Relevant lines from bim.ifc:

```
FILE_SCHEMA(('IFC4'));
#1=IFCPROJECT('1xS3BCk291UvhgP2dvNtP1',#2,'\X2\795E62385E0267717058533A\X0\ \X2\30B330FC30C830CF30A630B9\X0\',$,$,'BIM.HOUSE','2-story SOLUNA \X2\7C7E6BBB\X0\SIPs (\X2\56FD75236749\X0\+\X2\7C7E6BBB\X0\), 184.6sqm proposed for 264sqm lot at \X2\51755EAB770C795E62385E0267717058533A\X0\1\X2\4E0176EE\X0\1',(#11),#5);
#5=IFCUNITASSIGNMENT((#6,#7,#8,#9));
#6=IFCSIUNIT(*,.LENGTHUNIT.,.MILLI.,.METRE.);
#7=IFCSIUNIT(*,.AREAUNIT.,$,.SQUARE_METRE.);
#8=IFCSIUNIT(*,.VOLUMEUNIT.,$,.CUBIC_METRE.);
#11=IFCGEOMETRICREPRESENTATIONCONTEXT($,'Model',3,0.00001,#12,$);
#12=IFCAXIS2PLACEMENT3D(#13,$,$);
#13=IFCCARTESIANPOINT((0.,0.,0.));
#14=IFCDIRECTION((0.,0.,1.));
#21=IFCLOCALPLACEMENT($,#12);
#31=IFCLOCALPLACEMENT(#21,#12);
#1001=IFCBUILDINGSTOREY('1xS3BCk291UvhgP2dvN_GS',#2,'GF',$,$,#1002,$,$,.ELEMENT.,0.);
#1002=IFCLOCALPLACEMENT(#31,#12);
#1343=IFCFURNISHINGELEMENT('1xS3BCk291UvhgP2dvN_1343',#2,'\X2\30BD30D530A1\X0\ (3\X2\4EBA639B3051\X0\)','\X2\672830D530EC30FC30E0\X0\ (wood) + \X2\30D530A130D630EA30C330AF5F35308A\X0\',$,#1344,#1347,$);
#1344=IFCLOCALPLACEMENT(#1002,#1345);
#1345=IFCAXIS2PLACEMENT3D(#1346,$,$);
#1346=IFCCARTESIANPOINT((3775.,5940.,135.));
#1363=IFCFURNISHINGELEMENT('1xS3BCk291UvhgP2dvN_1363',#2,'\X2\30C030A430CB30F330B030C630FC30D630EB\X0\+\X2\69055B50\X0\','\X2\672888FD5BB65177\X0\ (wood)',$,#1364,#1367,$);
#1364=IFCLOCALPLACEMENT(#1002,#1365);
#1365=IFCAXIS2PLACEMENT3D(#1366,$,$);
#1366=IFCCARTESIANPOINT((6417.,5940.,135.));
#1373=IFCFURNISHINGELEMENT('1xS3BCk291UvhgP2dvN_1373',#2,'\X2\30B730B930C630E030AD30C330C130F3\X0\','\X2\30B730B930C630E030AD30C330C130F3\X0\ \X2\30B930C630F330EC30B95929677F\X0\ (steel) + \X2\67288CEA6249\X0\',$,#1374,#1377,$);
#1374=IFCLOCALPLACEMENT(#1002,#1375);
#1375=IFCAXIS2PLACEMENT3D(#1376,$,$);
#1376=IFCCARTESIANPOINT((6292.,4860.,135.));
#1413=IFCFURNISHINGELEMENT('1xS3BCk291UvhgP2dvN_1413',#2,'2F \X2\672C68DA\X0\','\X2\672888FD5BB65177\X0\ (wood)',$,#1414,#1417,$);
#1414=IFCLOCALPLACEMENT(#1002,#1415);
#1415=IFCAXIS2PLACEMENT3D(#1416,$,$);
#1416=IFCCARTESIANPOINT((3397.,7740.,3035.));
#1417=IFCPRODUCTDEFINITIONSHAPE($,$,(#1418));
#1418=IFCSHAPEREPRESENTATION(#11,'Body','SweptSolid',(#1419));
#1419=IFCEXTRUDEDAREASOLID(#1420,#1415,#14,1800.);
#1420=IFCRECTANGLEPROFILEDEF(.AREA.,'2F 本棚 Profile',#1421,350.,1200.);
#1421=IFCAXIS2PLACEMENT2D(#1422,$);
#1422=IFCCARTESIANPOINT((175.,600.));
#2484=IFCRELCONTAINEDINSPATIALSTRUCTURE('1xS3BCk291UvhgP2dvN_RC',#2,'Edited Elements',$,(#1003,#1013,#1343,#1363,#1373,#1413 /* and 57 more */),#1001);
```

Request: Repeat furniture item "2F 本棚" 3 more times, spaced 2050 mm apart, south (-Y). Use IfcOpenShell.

```python
import numpy as np
import ifcopenshell
import ifcopenshell.api.geometry
import ifcopenshell.api.root
import ifcopenshell.util.element
import ifcopenshell.util.placement
import ifcopenshell.util.unit

model = ifcopenshell.open("bim.ifc")
unit_scale = ifcopenshell.util.unit.calculate_unit_scale(model)


def reuse_history(source, copy):
    """copy_class also copies each property set's owner history, people and application; keep the originals."""
    for rel in copy.IsDefinedBy:
        if rel.is_a("IfcRelDefinesByProperties") and (history := rel.RelatingPropertyDefinition.OwnerHistory):
            rel.RelatingPropertyDefinition.OwnerHistory = source.OwnerHistory
            ifcopenshell.util.element.remove_deep2(model, history)


source = model.by_guid("1xS3BCk291UvhgP2dvN_1413")
base = ifcopenshell.util.placement.get_local_placement(source.ObjectPlacement)
step = np.array([0.0, -1.0, 0.0]) * 2.05 / unit_scale

for i in range(1, 4):
    copy = ifcopenshell.api.root.copy_class(model, product=source)
    copy.Representation = ifcopenshell.util.element.copy_deep(
        model, source.Representation, exclude=["IfcGeometricRepresentationContext", "IfcRepresentationMap"]
    )
    reuse_history(source, copy)
    matrix = base.copy()
    matrix[:3, 3] += i * step
    print("added at", matrix[:3, 3].round(3) + 0.0)
    ifcopenshell.api.geometry.edit_object_placement(model, product=copy, matrix=matrix, is_si=False)

model.write("bim-out.ifc")
```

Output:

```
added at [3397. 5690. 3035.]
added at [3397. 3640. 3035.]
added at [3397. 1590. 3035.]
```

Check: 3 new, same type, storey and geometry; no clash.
